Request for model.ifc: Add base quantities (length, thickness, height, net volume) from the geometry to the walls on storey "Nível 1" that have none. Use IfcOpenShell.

First a look at what the model holds.

```python
import ifcopenshell
import ifcopenshell.util.element
import ifcopenshell.util.unit

model = ifcopenshell.open("model.ifc")
print(model.schema)
for unit_type in ("LENGTHUNIT", "AREAUNIT", "VOLUMEUNIT"):
    print(unit_type, ifcopenshell.util.unit.calculate_unit_scale(model, unit_type))
storey = next(s for s in model.by_type("IfcBuildingStorey") if s.Name == "Nível 1")
walls = [e for e in ifcopenshell.util.element.get_decomposition(storey) if e.is_a("IfcWall")]
for e in sorted(walls, key=lambda e: e.id()):
    print(e.id(), e.is_a(), e.Name, list(ifcopenshell.util.element.get_psets(e, qtos_only=True)), sep=" | ")
```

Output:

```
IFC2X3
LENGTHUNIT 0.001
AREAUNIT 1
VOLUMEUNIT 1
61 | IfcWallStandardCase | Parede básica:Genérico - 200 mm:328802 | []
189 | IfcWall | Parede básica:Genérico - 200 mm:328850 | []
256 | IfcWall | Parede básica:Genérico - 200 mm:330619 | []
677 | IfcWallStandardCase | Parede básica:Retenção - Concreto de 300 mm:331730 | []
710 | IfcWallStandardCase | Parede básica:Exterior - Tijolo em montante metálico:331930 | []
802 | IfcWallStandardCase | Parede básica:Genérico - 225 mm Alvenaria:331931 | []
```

```python
import ifcopenshell
import ifcopenshell.api.pset
import ifcopenshell.geom
import ifcopenshell.util.element
import ifcopenshell.util.shape
import ifcopenshell.util.unit

model = ifcopenshell.open("model.ifc")
unit_scale = ifcopenshell.util.unit.calculate_unit_scale(model)
volume_scale = ifcopenshell.util.unit.calculate_unit_scale(model, "VOLUMEUNIT")
settings = ifcopenshell.geom.settings()

storey = next(s for s in model.by_type("IfcBuildingStorey") if s.Name == "Nível 1")
walls = [e for e in ifcopenshell.util.element.get_decomposition(storey) if e.is_a("IfcWall")]

for e in sorted(walls, key=lambda e: e.id()):
    if ifcopenshell.util.element.get_psets(e, qtos_only=True, should_inherit=False):
        continue
    # Geometry comes back in metres, in the element's own axes.
    shape = ifcopenshell.geom.create_shape(settings, e)
    values = {
        "Length": ifcopenshell.util.shape.get_x(shape.geometry) / unit_scale,
        "Width": ifcopenshell.util.shape.get_y(shape.geometry) / unit_scale,
        "Height": ifcopenshell.util.shape.get_z(shape.geometry) / unit_scale,
        "NetVolume": ifcopenshell.util.shape.get_volume(shape.geometry) / volume_scale,
    }
    qto = ifcopenshell.api.pset.add_qto(model, product=e, name="BaseQuantities")
    ifcopenshell.api.pset.edit_qto(model, qto=qto, properties=values)
    print(e.id(), {k: round(v, 3) for k, v in values.items()})

model.write("model_rev.ifc")
```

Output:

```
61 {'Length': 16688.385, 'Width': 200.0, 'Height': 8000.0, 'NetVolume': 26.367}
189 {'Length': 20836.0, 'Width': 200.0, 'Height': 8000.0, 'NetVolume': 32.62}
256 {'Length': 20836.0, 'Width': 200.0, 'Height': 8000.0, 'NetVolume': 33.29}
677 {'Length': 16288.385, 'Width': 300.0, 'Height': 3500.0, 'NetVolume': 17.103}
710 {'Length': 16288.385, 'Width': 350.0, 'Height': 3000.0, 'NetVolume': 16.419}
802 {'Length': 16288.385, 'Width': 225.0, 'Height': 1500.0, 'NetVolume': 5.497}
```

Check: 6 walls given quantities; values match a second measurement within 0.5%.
